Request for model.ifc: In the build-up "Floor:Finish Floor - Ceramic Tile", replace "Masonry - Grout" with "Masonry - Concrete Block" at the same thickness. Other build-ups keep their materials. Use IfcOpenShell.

First a look at what the model holds.

```python
import ifcopenshell
import ifcopenshell.util.element

model = ifcopenshell.open("model.ifc")
print(model.schema)
for layer_set in model.by_type("IfcMaterialLayerSet"):
    if layer_set.LayerSetName == "Floor:Finish Floor - Ceramic Tile":
        for layer in layer_set.MaterialLayers:
            print(layer.id(), layer.Material and layer.Material.Name, layer.LayerThickness, sep=" | ")
        print(len(ifcopenshell.util.element.get_elements_by_material(model, layer_set)), "elements and types use it")
print(sorted(m.Name for m in model.by_type("IfcMaterial") if m.Name)[:60])
```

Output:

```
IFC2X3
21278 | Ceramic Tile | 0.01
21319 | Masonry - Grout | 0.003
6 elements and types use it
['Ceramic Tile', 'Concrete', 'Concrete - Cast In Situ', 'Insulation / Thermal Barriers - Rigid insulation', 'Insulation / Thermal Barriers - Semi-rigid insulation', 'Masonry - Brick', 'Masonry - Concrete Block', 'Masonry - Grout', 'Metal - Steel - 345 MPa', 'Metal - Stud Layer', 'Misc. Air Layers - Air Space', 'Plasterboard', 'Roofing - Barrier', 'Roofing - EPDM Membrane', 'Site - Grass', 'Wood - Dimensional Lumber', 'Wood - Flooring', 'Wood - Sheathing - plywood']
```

```python
import ifcopenshell
import ifcopenshell.api.material

model = ifcopenshell.open("model.ifc")

layer_set = next(s for s in model.by_type("IfcMaterialLayerSet") if s.LayerSetName == "Floor:Finish Floor - Ceramic Tile")
layer = next(l for l in layer_set.MaterialLayers if l.Material and l.Material.Name == "Masonry - Grout")
material = next(m for m in model.by_type("IfcMaterial") if m.Name == "Masonry - Concrete Block")

# Point this one layer at the other material; renaming the old one would change it everywhere.
ifcopenshell.api.material.edit_layer(model, layer=layer, attributes={}, material=material)

print([l.Material.Name if l.Material else None for l in layer_set.MaterialLayers])

model.write("model_edited.ifc")
```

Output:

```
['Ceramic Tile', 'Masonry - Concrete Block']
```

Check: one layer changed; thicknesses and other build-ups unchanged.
